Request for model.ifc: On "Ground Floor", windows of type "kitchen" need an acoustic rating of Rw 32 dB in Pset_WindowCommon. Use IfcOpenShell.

First a look at what the model holds.

```python
import ifcopenshell
import ifcopenshell.util.element

model = ifcopenshell.open("model.ifc")
print(model.schema)
storey = next(s for s in model.by_type("IfcBuildingStorey") if s.Name == "Ground Floor")
windows = [e for e in ifcopenshell.util.element.get_decomposition(storey) if e.is_a("IfcWindow")]
seen = {}
for e in windows:
    element_type = ifcopenshell.util.element.get_type(e)
    key = (element_type.Name if element_type != e and element_type else None, ifcopenshell.util.element.get_pset(e, "Pset_WindowCommon", "AcousticRating"))
    seen[key] = seen.get(key, 0) + 1
for (name, value), count in sorted(seen.items(), key=str):
    print(count, "x", name, "|", value)
```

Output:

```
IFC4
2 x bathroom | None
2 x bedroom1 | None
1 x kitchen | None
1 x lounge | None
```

```python
import ifcopenshell
import ifcopenshell.api.pset
import ifcopenshell.util.element

model = ifcopenshell.open("model.ifc")

storey = next(s for s in model.by_type("IfcBuildingStorey") if s.Name == "Ground Floor")
windows = [e for e in ifcopenshell.util.element.get_decomposition(storey) if e.is_a("IfcWindow")]

count = 0
for e in windows:
    element_type = ifcopenshell.util.element.get_type(e)
    if element_type in (None, e) or element_type.Name != "kitchen":
        continue
    # add_pset returns the element's existing set when there is one.
    pset = ifcopenshell.api.pset.add_pset(model, product=e, name="Pset_WindowCommon")
    ifcopenshell.api.pset.edit_pset(model, pset=pset, properties={"AcousticRating": "Rw 32 dB"})
    count += 1

print(count, "windows updated")

model.write("model_v2.ifc")
```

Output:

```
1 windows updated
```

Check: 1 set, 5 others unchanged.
